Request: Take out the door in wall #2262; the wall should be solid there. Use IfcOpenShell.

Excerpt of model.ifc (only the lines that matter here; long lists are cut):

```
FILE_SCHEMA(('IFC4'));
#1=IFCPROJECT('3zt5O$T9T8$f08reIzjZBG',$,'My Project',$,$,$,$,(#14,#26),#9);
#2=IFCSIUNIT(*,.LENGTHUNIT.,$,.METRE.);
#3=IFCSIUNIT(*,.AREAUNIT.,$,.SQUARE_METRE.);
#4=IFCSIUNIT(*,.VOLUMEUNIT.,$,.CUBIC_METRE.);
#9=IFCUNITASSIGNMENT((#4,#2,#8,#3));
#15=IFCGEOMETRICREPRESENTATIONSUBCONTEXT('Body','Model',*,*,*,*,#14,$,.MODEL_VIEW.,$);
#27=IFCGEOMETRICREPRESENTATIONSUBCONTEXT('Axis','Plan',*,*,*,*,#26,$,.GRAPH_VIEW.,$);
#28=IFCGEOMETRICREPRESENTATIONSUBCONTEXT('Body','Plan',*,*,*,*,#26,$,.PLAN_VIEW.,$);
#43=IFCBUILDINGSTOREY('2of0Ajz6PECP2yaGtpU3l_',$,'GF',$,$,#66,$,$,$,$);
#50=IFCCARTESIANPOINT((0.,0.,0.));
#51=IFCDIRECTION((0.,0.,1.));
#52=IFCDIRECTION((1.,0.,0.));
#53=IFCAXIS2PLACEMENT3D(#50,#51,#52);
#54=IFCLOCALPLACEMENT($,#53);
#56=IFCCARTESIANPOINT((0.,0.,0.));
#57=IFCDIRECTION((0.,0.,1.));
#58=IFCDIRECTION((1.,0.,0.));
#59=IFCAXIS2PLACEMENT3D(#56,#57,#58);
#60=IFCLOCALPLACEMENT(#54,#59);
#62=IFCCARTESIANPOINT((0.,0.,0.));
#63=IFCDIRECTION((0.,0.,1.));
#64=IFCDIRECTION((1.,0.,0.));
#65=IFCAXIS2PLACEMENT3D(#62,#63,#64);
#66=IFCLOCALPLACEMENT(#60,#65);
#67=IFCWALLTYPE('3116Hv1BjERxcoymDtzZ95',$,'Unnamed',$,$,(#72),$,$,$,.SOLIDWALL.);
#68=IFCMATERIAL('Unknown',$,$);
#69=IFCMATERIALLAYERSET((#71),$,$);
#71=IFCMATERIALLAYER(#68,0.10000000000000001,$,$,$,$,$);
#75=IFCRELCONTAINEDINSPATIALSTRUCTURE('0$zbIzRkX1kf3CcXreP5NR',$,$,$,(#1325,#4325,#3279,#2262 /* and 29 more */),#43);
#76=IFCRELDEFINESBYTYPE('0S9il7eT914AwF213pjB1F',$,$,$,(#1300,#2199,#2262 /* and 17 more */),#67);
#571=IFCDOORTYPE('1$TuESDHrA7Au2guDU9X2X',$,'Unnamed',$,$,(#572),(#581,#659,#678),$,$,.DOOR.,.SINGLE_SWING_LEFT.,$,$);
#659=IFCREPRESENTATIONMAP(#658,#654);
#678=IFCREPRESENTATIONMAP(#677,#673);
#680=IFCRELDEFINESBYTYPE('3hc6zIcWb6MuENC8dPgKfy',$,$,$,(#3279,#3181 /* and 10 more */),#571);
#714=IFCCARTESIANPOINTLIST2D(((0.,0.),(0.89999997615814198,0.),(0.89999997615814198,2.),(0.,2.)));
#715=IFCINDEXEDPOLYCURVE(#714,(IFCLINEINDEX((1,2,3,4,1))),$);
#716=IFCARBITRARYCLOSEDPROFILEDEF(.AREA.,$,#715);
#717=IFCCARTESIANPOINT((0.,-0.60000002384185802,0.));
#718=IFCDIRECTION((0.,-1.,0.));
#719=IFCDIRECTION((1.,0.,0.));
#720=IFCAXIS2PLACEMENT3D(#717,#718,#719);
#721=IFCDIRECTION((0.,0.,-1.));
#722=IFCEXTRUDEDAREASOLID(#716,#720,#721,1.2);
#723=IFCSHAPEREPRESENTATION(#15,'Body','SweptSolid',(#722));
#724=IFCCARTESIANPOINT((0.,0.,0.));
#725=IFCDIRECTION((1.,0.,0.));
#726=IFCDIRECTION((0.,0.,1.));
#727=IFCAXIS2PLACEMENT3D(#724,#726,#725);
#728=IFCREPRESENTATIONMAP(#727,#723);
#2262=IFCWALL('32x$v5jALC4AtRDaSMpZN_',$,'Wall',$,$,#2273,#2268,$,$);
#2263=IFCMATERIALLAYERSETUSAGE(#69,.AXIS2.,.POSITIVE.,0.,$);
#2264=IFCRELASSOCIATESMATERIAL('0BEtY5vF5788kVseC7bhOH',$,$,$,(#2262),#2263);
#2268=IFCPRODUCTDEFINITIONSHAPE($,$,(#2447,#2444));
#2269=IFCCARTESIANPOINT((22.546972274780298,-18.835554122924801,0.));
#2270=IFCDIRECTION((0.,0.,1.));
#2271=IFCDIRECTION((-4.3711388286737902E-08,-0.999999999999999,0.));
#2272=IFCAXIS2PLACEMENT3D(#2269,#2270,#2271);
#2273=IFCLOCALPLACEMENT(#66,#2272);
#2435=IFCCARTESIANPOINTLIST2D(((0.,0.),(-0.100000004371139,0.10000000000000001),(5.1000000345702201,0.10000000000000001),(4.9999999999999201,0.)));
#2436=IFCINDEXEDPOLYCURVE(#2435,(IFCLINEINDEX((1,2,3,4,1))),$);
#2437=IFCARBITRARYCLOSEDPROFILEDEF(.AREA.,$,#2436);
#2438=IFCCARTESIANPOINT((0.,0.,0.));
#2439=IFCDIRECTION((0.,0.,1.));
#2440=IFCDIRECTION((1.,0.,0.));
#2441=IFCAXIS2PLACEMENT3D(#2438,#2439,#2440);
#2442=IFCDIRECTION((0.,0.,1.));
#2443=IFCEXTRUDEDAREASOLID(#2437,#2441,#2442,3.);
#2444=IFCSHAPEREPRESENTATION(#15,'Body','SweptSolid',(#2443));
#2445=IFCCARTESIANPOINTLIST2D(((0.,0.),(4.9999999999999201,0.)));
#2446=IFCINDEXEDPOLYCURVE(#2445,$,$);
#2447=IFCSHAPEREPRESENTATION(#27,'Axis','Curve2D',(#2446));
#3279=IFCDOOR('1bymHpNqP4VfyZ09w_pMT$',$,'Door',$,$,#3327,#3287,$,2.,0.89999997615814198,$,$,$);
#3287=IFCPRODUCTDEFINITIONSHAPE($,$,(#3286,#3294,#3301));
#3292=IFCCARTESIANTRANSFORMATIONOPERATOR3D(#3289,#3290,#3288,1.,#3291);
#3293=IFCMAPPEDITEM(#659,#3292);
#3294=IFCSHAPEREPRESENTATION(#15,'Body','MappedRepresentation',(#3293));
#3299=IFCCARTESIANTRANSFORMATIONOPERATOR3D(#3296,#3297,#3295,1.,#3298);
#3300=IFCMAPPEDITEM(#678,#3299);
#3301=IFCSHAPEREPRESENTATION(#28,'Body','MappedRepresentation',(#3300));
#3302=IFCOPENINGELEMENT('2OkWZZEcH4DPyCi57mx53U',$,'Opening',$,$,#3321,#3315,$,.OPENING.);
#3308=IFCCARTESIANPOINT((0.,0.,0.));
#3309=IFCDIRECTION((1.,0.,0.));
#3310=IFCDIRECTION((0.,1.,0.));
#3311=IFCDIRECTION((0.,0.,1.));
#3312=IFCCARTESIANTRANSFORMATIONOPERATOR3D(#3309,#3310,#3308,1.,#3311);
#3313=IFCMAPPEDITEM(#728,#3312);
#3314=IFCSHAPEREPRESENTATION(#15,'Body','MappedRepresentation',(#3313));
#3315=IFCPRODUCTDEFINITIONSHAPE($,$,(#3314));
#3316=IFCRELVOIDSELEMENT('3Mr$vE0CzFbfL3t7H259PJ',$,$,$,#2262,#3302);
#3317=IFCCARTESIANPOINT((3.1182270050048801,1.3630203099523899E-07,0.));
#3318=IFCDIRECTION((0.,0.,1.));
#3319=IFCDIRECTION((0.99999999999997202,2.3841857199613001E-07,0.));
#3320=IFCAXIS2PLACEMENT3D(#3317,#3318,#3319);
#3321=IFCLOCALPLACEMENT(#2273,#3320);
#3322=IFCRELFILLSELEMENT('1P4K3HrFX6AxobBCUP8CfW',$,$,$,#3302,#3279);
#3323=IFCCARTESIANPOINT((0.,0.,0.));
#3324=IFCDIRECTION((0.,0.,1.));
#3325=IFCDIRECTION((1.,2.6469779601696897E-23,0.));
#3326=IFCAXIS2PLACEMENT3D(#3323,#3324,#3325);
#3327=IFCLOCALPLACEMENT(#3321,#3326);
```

```python
import ifcopenshell
import ifcopenshell.api.feature
import ifcopenshell.api.root
import ifcopenshell.geom
import ifcopenshell.util.shape

model = ifcopenshell.open("model.ifc")
settings = ifcopenshell.geom.settings()


def volume(element):
    """Net volume in cubic metres, openings subtracted."""
    shape = ifcopenshell.geom.create_shape(settings, element)
    return ifcopenshell.util.shape.get_volume(shape.geometry)


door = model.by_guid("1bymHpNqP4VfyZ09w_pMT$")
opening = door.FillsVoids[0].RelatingOpeningElement
wall = opening.VoidsElements[0].RelatingBuildingElement
before = volume(wall)

ifcopenshell.api.root.remove_product(model, product=door)
ifcopenshell.api.feature.remove_feature(model, feature=opening)

after = volume(wall)

print(f"wall volume {before:.3f} -> {after:.3f} m3")

model.write("model_edited.ifc")
```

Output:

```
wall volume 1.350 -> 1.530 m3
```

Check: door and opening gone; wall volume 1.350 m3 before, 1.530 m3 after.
